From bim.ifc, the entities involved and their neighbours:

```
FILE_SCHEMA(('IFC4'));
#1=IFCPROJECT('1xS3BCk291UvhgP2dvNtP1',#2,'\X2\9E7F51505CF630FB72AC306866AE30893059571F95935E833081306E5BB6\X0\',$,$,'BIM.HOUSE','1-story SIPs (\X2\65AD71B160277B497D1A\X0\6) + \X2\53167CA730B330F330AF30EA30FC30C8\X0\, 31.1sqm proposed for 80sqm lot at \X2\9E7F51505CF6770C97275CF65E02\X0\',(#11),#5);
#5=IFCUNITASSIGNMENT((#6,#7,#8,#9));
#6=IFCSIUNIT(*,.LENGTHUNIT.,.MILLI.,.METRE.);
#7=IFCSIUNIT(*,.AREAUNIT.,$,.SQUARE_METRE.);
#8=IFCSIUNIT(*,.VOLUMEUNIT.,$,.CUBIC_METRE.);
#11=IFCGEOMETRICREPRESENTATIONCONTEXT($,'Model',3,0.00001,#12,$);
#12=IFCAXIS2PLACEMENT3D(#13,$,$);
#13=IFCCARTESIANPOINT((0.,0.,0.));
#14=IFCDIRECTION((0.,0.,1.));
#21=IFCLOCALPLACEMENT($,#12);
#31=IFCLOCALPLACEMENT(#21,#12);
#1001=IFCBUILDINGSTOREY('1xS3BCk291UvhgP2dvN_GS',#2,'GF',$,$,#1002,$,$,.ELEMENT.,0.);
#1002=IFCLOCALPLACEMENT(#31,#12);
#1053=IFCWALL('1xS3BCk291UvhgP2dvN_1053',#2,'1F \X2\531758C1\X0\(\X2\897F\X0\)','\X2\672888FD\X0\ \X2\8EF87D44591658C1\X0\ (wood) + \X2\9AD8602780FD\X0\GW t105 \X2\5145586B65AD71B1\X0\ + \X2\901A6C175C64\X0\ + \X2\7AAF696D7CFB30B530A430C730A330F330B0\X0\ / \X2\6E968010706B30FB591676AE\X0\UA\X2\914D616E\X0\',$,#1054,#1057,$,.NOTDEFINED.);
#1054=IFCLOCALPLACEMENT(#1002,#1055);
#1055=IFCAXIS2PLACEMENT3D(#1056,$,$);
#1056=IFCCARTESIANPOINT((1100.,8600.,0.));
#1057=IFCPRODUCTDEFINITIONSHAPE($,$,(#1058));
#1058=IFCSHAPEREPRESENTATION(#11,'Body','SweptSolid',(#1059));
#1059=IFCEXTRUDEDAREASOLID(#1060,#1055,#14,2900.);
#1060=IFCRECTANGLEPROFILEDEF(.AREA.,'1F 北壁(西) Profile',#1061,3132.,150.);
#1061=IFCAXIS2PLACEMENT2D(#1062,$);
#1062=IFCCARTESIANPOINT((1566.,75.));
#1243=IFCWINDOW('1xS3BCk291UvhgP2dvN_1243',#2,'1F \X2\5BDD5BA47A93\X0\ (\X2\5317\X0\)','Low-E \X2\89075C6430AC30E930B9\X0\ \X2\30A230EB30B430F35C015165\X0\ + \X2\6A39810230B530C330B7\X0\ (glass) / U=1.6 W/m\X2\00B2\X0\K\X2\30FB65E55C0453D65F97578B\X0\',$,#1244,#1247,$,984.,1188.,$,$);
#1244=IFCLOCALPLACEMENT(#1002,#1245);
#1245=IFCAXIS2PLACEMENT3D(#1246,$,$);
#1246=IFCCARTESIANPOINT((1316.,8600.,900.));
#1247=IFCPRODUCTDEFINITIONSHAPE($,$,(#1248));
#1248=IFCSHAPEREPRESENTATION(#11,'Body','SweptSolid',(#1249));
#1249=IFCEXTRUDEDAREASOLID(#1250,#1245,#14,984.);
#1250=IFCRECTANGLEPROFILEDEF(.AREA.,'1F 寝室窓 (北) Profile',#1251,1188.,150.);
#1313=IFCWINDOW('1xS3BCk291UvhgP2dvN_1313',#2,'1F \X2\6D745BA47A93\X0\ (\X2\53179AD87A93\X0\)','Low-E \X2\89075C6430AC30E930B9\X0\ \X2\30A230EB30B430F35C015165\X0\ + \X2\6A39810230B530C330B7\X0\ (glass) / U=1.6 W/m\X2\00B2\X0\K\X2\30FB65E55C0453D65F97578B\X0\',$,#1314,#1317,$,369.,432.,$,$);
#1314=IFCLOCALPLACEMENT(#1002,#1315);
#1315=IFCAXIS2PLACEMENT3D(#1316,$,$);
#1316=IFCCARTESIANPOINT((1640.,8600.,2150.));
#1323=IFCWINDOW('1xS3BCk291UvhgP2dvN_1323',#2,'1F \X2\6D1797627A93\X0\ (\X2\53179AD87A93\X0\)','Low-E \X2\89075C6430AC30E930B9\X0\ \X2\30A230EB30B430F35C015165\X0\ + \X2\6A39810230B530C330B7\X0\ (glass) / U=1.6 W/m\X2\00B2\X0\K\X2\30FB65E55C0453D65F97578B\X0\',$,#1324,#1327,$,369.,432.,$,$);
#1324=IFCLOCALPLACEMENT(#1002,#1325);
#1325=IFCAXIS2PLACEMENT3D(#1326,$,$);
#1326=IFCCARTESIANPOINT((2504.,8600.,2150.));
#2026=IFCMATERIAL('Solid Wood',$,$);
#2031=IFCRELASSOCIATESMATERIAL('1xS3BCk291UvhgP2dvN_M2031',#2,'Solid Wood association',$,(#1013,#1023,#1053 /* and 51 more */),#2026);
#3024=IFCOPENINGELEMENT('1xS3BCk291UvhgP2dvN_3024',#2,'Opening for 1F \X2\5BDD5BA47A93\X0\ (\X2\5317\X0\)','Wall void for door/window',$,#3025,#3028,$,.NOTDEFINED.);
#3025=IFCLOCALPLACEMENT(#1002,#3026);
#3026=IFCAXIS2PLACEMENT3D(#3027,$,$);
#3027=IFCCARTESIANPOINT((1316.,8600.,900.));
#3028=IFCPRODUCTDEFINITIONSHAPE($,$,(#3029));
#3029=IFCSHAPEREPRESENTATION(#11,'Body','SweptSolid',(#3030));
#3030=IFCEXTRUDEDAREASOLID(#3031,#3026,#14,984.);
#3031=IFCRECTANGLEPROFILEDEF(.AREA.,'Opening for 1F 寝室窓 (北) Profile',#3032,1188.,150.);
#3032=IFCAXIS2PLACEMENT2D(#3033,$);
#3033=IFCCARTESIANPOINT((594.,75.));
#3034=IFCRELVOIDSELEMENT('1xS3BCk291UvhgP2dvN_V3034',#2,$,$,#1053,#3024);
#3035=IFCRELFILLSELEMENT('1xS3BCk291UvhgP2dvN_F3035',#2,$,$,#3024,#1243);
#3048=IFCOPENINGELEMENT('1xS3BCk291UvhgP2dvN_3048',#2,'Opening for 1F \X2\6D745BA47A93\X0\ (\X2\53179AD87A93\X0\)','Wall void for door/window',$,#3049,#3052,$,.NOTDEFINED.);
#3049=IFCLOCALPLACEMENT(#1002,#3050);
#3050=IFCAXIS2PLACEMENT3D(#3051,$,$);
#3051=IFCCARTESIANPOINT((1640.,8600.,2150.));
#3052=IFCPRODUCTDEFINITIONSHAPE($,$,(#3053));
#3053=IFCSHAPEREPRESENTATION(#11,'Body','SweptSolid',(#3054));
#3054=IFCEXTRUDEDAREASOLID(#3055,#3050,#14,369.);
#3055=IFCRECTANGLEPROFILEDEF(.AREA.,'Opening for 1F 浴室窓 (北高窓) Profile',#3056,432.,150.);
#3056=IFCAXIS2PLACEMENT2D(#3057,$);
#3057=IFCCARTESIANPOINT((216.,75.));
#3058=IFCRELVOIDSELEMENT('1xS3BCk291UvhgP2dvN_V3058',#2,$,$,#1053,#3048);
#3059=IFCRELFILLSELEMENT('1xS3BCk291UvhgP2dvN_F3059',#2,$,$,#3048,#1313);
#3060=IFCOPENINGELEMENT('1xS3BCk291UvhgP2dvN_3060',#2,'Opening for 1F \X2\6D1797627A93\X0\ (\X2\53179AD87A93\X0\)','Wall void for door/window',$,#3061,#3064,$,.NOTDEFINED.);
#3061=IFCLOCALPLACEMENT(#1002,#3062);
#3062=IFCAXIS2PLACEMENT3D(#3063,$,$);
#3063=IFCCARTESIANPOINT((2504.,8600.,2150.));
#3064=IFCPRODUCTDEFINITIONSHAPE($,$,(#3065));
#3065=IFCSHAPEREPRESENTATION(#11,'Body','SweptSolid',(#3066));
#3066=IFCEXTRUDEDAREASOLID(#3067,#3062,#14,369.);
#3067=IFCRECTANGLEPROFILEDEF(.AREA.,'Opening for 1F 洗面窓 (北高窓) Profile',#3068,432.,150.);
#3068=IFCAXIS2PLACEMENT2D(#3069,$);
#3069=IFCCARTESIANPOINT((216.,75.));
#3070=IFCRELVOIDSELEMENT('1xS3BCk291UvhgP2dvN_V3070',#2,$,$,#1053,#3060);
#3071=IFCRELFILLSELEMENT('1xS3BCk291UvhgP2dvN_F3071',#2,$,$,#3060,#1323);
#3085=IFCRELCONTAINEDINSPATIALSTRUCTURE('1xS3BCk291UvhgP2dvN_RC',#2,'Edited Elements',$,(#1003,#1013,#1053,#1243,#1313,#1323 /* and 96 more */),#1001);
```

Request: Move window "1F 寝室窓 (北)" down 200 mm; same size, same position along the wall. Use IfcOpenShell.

```python
import numpy as np
import ifcopenshell
import ifcopenshell.api.geometry
import ifcopenshell.util.placement
import ifcopenshell.util.unit

model = ifcopenshell.open("bim.ifc")
unit_scale = ifcopenshell.util.unit.calculate_unit_scale(model)

window = model.by_id(1243)
opening = window.FillsVoids[0].RelatingOpeningElement
dz = -200.0

shift = np.array([0.0, 0.0, dz])
# The window is not placed relative to its opening, so move both.
for product in (opening, window):
    matrix = ifcopenshell.util.placement.get_local_placement(product.ObjectPlacement)
    matrix[:3, 3] += shift
    ifcopenshell.api.geometry.edit_object_placement(model, product=product, matrix=matrix, is_si=False)

print(f"moved by {dz * unit_scale:+.3f} m")

model.write("bim_rev.ifc")
```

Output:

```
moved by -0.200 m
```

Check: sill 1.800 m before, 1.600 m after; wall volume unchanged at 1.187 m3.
